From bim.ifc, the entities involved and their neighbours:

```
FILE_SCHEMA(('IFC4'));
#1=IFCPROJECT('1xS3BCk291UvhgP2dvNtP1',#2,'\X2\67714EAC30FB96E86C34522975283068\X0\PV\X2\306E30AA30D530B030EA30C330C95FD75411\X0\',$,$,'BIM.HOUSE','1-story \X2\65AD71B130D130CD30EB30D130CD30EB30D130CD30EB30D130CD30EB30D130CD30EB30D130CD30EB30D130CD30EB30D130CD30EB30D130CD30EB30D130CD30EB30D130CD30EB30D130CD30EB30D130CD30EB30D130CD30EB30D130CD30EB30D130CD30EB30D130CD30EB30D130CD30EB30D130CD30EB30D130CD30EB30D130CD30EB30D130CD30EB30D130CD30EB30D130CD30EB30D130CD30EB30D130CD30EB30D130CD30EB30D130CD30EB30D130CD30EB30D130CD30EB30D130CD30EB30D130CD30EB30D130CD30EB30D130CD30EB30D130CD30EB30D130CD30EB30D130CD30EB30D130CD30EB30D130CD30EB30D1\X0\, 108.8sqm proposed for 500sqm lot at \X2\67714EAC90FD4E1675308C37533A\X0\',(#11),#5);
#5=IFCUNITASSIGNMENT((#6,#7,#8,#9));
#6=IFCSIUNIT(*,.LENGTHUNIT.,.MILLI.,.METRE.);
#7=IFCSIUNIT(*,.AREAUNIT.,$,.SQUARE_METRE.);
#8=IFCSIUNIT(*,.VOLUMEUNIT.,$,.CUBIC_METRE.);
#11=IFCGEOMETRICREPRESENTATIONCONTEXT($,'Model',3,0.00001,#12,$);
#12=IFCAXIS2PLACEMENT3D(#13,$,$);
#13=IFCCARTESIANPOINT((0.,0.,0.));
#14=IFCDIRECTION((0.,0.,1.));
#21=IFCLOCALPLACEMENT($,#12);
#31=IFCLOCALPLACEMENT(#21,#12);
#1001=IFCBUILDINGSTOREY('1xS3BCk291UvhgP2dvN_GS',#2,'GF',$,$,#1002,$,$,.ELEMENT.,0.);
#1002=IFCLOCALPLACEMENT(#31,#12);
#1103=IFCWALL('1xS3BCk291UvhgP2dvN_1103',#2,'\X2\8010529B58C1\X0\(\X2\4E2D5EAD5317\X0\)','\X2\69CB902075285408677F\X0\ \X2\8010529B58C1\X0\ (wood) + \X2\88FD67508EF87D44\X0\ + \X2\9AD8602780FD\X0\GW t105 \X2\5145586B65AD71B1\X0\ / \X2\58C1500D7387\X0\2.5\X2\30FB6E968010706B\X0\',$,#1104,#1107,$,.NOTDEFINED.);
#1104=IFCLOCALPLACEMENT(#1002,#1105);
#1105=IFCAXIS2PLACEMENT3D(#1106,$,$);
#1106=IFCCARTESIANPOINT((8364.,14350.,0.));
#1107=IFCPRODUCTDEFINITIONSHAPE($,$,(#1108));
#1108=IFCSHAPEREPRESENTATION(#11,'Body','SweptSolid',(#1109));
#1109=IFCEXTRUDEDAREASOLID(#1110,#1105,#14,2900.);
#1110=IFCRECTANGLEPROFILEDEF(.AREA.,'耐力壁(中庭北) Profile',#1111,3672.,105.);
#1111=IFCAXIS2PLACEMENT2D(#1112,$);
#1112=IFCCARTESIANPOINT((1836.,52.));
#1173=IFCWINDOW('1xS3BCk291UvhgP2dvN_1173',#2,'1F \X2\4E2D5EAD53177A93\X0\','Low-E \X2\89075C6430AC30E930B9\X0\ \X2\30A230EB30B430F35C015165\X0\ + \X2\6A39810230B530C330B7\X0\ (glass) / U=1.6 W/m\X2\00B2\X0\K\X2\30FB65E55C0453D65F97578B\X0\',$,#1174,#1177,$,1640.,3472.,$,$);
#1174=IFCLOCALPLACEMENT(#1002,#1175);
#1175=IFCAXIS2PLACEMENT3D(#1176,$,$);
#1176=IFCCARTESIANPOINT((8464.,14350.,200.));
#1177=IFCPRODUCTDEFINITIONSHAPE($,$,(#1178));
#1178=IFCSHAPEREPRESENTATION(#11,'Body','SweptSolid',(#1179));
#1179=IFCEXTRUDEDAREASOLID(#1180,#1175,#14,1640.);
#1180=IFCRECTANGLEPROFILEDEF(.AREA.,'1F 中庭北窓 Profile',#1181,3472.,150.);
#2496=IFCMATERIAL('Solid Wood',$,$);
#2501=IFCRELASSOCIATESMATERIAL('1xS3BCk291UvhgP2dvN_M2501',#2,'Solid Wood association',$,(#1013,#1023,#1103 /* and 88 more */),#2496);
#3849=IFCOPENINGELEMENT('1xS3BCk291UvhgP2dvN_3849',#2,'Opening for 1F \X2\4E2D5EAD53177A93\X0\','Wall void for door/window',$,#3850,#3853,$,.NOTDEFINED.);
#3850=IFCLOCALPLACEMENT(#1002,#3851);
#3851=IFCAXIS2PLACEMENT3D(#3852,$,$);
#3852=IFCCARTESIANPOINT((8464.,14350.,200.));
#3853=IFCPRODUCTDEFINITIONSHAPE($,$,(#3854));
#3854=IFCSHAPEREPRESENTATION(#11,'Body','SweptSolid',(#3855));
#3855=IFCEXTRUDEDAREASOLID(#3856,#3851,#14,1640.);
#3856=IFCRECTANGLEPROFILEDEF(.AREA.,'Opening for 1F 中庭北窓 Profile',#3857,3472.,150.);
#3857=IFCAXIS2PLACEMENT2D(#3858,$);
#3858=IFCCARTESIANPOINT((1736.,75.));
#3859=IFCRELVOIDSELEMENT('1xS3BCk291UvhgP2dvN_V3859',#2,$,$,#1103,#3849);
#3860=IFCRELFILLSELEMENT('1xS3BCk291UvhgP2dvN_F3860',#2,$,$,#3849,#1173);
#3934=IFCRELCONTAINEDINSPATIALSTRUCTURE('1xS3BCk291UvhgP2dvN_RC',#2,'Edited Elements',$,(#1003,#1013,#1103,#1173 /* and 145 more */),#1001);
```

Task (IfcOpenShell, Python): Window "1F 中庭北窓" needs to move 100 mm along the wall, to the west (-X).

```python
import ifcopenshell
import ifcopenshell.api.geometry
import ifcopenshell.util.placement
import ifcopenshell.util.unit

model = ifcopenshell.open("bim.ifc")
unit_scale = ifcopenshell.util.unit.calculate_unit_scale(model)

window = model.by_id(1173)
opening = window.FillsVoids[0].RelatingOpeningElement
wall = opening.VoidsElements[0].RelatingBuildingElement

wall_matrix = ifcopenshell.util.placement.get_local_placement(wall.ObjectPlacement)
shift = wall_matrix[:3, 0] * -0.1 / unit_scale
before = ifcopenshell.util.placement.get_local_placement(window.ObjectPlacement)[:3, 3].copy()

# The window is not placed relative to its opening, so move both.
for product in (opening, window):
    matrix = ifcopenshell.util.placement.get_local_placement(product.ObjectPlacement)
    matrix[:3, 3] += shift
    ifcopenshell.api.geometry.edit_object_placement(model, product=product, matrix=matrix, is_si=False)

after = ifcopenshell.util.placement.get_local_placement(window.ObjectPlacement)[:3, 3]
print("window moved by", (after - before).round(3) + 0.0)

model.write("bim_v2.ifc")
```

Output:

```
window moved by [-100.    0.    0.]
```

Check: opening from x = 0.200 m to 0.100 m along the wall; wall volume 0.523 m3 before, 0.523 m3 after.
